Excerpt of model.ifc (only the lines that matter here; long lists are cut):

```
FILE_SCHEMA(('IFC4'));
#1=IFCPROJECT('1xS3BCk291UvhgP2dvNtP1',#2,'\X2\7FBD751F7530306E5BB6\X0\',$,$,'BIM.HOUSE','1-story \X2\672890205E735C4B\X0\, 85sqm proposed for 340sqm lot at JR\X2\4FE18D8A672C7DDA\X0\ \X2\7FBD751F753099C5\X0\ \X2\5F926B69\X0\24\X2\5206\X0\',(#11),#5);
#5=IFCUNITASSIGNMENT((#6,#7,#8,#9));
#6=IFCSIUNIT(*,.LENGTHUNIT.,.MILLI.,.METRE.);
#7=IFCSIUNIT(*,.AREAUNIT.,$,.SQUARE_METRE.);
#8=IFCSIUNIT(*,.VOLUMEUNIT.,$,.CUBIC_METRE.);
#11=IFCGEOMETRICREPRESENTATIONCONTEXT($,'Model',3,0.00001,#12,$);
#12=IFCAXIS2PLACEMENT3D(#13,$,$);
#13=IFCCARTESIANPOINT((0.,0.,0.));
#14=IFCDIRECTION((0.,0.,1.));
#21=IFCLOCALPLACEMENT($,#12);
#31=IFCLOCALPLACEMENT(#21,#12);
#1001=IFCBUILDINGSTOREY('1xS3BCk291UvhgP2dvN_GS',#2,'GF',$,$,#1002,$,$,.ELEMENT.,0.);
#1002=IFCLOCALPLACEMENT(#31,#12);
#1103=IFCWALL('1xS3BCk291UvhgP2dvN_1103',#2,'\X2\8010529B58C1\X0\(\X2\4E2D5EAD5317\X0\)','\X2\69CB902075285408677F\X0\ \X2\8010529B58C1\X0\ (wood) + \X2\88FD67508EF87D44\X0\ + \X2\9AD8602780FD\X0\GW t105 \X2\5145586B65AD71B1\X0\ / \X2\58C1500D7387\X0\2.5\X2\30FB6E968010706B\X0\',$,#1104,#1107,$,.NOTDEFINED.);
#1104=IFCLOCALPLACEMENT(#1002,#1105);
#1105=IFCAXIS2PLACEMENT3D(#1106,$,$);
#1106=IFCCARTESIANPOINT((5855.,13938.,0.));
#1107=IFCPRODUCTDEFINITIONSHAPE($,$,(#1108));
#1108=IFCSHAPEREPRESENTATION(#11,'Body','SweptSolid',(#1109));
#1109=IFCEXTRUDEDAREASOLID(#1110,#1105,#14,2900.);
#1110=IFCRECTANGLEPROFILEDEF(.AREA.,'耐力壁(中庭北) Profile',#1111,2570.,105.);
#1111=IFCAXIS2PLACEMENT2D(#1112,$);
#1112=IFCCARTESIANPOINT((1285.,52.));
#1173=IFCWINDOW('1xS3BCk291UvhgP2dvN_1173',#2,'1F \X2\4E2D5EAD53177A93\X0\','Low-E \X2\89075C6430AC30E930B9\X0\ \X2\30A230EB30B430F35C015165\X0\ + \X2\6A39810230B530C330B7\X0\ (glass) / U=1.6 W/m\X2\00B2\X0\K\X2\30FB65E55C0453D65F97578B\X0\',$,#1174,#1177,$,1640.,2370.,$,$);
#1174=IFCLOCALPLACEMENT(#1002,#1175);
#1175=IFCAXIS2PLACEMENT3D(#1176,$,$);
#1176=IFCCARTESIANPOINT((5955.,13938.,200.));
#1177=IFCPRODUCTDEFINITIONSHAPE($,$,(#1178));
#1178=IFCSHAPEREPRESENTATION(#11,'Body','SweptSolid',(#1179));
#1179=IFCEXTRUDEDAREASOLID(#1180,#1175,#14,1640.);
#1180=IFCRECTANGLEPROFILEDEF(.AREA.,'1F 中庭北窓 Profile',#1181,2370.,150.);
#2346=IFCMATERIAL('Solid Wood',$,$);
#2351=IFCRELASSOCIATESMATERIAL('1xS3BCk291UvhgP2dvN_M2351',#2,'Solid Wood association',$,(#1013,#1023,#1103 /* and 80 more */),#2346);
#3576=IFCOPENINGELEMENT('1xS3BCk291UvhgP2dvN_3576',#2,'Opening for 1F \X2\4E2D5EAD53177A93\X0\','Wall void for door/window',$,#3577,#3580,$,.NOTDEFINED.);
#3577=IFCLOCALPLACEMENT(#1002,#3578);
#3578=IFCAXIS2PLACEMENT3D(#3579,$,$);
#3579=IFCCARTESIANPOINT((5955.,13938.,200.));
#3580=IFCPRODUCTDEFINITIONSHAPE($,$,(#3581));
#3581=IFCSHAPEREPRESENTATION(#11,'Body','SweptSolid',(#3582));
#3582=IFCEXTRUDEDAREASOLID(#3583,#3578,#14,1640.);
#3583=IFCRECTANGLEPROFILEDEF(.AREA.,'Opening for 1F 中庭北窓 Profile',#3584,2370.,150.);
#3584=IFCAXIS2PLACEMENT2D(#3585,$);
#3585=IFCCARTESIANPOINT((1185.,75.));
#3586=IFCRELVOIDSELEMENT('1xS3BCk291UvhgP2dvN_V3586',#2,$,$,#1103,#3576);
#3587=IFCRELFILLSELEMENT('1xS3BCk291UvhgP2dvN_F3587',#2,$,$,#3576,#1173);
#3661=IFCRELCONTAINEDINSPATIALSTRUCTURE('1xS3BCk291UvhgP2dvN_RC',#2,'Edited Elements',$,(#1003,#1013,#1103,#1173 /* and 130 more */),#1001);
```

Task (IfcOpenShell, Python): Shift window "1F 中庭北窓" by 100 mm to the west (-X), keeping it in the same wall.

```python
import ifcopenshell
import ifcopenshell.api.geometry
import ifcopenshell.util.placement

model = ifcopenshell.open("model.ifc")

window = model.by_guid("1xS3BCk291UvhgP2dvN_1173")
opening = window.FillsVoids[0].RelatingOpeningElement
wall = opening.VoidsElements[0].RelatingBuildingElement

wall_matrix = ifcopenshell.util.placement.get_local_placement(wall.ObjectPlacement)
shift = wall_matrix[:3, 0] * -100.0
before = ifcopenshell.util.placement.get_local_placement(window.ObjectPlacement)[:3, 3].copy()

# The window is not placed relative to its opening, so move both.
for product in (opening, window):
    matrix = ifcopenshell.util.placement.get_local_placement(product.ObjectPlacement)
    matrix[:3, 3] += shift
    ifcopenshell.api.geometry.edit_object_placement(model, product=product, matrix=matrix, is_si=False)

after = ifcopenshell.util.placement.get_local_placement(window.ObjectPlacement)[:3, 3]
print("window moved by", (after - before).round(3) + 0.0)

model.write("model-out.ifc")
```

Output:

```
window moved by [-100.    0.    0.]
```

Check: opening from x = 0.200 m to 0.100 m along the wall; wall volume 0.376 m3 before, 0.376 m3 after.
